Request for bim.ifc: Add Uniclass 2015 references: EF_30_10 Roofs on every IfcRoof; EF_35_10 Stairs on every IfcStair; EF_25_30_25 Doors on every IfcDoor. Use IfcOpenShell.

First a look at what the model holds.

```python
import ifcopenshell

model = ifcopenshell.open("bim.ifc")
print(model.schema)
print("classifications:", [c.Name for c in model.by_type("IfcClassification")])
for ifc_class in ("IfcDoor", "IfcRoof", "IfcStair", "IfcWall", "IfcWindow"):
    print(ifc_class, len(model.by_type(ifc_class)))
```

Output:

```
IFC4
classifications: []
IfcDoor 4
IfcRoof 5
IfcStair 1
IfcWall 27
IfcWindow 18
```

```python
import ifcopenshell
import ifcopenshell.api.classification

model = ifcopenshell.open("bim.ifc")

system = ifcopenshell.api.classification.add_classification(model, classification="Uniclass 2015")

codes = {
    "IfcRoof": ("EF_30_10", "Roofs"),
    "IfcStair": ("EF_35_10", "Stairs"),
    "IfcDoor": ("EF_25_30_25", "Doors"),
}
for ifc_class, (code, name) in codes.items():
    products = model.by_type(ifc_class)
    ifcopenshell.api.classification.add_reference(
        model, products=products, classification=system, identification=code, name=name
    )
    print(code, len(products))

model.write("bim_updated.ifc")
```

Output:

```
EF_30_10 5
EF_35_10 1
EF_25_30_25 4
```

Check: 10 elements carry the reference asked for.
